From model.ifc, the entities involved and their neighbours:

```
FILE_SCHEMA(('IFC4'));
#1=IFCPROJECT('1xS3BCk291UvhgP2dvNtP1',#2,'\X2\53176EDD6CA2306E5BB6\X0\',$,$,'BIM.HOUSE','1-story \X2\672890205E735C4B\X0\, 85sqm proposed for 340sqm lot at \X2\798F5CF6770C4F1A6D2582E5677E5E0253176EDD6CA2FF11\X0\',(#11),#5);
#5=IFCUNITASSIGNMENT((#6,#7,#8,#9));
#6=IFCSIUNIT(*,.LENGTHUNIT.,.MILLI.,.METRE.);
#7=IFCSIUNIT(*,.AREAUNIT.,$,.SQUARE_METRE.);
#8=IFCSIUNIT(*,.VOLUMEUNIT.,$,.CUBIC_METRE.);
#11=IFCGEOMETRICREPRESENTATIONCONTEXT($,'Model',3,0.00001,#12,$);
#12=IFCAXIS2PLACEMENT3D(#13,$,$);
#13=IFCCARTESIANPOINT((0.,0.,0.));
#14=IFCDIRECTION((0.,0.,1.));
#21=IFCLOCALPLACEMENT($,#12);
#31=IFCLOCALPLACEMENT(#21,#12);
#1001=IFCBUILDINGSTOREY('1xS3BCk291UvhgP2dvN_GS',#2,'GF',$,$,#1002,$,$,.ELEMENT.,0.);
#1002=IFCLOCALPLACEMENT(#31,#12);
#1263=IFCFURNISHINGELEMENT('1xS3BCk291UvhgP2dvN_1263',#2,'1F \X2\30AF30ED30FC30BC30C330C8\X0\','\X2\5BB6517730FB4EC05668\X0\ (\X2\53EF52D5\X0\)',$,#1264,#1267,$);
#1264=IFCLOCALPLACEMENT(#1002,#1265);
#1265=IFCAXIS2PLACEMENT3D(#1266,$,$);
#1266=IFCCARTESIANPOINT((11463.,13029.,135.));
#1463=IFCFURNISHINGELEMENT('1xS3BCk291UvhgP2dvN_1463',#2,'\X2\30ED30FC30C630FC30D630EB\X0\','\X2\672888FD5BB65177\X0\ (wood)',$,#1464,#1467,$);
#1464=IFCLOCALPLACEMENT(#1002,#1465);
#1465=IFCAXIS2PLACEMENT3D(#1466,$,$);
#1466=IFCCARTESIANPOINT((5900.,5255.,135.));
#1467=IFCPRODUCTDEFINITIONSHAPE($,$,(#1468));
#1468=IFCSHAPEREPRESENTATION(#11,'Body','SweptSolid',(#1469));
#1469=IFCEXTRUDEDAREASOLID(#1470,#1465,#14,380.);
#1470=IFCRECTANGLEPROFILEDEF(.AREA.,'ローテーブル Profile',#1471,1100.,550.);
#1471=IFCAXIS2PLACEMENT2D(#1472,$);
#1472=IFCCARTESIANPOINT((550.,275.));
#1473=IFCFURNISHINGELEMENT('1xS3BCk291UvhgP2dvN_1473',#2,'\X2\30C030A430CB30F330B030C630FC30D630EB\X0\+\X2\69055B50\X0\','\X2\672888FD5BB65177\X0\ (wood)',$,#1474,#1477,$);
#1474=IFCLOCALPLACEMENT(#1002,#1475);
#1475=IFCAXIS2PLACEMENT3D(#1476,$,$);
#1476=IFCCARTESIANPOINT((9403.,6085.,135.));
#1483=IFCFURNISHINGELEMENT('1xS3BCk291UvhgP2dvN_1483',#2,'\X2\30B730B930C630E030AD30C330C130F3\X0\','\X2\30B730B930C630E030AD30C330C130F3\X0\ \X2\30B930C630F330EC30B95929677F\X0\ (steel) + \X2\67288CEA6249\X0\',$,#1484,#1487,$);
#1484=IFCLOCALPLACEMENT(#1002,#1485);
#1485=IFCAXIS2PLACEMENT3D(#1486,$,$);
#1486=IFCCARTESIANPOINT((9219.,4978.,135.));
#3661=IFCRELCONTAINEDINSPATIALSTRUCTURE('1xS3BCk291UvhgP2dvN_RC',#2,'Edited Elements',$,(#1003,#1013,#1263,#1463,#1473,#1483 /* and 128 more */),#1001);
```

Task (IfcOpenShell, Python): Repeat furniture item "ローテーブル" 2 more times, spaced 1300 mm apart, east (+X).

```python
import numpy as np
import ifcopenshell
import ifcopenshell.api.geometry
import ifcopenshell.api.root
import ifcopenshell.util.element
import ifcopenshell.util.placement

model = ifcopenshell.open("model.ifc")


def reuse_history(source, copy):
    """copy_class also copies each property set's owner history, people and application; keep the originals."""
    for rel in copy.IsDefinedBy:
        if rel.is_a("IfcRelDefinesByProperties") and (history := rel.RelatingPropertyDefinition.OwnerHistory):
            rel.RelatingPropertyDefinition.OwnerHistory = source.OwnerHistory
            ifcopenshell.util.element.remove_deep2(model, history)


source = model.by_guid("1xS3BCk291UvhgP2dvN_1463")
base = ifcopenshell.util.placement.get_local_placement(source.ObjectPlacement)
step = np.array([1.0, 0.0, 0.0]) * 1300.0

for i in range(1, 3):
    copy = ifcopenshell.api.root.copy_class(model, product=source)
    copy.Representation = ifcopenshell.util.element.copy_deep(
        model, source.Representation, exclude=["IfcGeometricRepresentationContext", "IfcRepresentationMap"]
    )
    reuse_history(source, copy)
    matrix = base.copy()
    matrix[:3, 3] += i * step
    print("added at", matrix[:3, 3].round(3) + 0.0)
    ifcopenshell.api.geometry.edit_object_placement(model, product=copy, matrix=matrix, is_si=False)

model.write("model_updated.ifc")
```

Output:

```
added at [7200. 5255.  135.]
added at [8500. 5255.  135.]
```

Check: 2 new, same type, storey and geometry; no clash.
